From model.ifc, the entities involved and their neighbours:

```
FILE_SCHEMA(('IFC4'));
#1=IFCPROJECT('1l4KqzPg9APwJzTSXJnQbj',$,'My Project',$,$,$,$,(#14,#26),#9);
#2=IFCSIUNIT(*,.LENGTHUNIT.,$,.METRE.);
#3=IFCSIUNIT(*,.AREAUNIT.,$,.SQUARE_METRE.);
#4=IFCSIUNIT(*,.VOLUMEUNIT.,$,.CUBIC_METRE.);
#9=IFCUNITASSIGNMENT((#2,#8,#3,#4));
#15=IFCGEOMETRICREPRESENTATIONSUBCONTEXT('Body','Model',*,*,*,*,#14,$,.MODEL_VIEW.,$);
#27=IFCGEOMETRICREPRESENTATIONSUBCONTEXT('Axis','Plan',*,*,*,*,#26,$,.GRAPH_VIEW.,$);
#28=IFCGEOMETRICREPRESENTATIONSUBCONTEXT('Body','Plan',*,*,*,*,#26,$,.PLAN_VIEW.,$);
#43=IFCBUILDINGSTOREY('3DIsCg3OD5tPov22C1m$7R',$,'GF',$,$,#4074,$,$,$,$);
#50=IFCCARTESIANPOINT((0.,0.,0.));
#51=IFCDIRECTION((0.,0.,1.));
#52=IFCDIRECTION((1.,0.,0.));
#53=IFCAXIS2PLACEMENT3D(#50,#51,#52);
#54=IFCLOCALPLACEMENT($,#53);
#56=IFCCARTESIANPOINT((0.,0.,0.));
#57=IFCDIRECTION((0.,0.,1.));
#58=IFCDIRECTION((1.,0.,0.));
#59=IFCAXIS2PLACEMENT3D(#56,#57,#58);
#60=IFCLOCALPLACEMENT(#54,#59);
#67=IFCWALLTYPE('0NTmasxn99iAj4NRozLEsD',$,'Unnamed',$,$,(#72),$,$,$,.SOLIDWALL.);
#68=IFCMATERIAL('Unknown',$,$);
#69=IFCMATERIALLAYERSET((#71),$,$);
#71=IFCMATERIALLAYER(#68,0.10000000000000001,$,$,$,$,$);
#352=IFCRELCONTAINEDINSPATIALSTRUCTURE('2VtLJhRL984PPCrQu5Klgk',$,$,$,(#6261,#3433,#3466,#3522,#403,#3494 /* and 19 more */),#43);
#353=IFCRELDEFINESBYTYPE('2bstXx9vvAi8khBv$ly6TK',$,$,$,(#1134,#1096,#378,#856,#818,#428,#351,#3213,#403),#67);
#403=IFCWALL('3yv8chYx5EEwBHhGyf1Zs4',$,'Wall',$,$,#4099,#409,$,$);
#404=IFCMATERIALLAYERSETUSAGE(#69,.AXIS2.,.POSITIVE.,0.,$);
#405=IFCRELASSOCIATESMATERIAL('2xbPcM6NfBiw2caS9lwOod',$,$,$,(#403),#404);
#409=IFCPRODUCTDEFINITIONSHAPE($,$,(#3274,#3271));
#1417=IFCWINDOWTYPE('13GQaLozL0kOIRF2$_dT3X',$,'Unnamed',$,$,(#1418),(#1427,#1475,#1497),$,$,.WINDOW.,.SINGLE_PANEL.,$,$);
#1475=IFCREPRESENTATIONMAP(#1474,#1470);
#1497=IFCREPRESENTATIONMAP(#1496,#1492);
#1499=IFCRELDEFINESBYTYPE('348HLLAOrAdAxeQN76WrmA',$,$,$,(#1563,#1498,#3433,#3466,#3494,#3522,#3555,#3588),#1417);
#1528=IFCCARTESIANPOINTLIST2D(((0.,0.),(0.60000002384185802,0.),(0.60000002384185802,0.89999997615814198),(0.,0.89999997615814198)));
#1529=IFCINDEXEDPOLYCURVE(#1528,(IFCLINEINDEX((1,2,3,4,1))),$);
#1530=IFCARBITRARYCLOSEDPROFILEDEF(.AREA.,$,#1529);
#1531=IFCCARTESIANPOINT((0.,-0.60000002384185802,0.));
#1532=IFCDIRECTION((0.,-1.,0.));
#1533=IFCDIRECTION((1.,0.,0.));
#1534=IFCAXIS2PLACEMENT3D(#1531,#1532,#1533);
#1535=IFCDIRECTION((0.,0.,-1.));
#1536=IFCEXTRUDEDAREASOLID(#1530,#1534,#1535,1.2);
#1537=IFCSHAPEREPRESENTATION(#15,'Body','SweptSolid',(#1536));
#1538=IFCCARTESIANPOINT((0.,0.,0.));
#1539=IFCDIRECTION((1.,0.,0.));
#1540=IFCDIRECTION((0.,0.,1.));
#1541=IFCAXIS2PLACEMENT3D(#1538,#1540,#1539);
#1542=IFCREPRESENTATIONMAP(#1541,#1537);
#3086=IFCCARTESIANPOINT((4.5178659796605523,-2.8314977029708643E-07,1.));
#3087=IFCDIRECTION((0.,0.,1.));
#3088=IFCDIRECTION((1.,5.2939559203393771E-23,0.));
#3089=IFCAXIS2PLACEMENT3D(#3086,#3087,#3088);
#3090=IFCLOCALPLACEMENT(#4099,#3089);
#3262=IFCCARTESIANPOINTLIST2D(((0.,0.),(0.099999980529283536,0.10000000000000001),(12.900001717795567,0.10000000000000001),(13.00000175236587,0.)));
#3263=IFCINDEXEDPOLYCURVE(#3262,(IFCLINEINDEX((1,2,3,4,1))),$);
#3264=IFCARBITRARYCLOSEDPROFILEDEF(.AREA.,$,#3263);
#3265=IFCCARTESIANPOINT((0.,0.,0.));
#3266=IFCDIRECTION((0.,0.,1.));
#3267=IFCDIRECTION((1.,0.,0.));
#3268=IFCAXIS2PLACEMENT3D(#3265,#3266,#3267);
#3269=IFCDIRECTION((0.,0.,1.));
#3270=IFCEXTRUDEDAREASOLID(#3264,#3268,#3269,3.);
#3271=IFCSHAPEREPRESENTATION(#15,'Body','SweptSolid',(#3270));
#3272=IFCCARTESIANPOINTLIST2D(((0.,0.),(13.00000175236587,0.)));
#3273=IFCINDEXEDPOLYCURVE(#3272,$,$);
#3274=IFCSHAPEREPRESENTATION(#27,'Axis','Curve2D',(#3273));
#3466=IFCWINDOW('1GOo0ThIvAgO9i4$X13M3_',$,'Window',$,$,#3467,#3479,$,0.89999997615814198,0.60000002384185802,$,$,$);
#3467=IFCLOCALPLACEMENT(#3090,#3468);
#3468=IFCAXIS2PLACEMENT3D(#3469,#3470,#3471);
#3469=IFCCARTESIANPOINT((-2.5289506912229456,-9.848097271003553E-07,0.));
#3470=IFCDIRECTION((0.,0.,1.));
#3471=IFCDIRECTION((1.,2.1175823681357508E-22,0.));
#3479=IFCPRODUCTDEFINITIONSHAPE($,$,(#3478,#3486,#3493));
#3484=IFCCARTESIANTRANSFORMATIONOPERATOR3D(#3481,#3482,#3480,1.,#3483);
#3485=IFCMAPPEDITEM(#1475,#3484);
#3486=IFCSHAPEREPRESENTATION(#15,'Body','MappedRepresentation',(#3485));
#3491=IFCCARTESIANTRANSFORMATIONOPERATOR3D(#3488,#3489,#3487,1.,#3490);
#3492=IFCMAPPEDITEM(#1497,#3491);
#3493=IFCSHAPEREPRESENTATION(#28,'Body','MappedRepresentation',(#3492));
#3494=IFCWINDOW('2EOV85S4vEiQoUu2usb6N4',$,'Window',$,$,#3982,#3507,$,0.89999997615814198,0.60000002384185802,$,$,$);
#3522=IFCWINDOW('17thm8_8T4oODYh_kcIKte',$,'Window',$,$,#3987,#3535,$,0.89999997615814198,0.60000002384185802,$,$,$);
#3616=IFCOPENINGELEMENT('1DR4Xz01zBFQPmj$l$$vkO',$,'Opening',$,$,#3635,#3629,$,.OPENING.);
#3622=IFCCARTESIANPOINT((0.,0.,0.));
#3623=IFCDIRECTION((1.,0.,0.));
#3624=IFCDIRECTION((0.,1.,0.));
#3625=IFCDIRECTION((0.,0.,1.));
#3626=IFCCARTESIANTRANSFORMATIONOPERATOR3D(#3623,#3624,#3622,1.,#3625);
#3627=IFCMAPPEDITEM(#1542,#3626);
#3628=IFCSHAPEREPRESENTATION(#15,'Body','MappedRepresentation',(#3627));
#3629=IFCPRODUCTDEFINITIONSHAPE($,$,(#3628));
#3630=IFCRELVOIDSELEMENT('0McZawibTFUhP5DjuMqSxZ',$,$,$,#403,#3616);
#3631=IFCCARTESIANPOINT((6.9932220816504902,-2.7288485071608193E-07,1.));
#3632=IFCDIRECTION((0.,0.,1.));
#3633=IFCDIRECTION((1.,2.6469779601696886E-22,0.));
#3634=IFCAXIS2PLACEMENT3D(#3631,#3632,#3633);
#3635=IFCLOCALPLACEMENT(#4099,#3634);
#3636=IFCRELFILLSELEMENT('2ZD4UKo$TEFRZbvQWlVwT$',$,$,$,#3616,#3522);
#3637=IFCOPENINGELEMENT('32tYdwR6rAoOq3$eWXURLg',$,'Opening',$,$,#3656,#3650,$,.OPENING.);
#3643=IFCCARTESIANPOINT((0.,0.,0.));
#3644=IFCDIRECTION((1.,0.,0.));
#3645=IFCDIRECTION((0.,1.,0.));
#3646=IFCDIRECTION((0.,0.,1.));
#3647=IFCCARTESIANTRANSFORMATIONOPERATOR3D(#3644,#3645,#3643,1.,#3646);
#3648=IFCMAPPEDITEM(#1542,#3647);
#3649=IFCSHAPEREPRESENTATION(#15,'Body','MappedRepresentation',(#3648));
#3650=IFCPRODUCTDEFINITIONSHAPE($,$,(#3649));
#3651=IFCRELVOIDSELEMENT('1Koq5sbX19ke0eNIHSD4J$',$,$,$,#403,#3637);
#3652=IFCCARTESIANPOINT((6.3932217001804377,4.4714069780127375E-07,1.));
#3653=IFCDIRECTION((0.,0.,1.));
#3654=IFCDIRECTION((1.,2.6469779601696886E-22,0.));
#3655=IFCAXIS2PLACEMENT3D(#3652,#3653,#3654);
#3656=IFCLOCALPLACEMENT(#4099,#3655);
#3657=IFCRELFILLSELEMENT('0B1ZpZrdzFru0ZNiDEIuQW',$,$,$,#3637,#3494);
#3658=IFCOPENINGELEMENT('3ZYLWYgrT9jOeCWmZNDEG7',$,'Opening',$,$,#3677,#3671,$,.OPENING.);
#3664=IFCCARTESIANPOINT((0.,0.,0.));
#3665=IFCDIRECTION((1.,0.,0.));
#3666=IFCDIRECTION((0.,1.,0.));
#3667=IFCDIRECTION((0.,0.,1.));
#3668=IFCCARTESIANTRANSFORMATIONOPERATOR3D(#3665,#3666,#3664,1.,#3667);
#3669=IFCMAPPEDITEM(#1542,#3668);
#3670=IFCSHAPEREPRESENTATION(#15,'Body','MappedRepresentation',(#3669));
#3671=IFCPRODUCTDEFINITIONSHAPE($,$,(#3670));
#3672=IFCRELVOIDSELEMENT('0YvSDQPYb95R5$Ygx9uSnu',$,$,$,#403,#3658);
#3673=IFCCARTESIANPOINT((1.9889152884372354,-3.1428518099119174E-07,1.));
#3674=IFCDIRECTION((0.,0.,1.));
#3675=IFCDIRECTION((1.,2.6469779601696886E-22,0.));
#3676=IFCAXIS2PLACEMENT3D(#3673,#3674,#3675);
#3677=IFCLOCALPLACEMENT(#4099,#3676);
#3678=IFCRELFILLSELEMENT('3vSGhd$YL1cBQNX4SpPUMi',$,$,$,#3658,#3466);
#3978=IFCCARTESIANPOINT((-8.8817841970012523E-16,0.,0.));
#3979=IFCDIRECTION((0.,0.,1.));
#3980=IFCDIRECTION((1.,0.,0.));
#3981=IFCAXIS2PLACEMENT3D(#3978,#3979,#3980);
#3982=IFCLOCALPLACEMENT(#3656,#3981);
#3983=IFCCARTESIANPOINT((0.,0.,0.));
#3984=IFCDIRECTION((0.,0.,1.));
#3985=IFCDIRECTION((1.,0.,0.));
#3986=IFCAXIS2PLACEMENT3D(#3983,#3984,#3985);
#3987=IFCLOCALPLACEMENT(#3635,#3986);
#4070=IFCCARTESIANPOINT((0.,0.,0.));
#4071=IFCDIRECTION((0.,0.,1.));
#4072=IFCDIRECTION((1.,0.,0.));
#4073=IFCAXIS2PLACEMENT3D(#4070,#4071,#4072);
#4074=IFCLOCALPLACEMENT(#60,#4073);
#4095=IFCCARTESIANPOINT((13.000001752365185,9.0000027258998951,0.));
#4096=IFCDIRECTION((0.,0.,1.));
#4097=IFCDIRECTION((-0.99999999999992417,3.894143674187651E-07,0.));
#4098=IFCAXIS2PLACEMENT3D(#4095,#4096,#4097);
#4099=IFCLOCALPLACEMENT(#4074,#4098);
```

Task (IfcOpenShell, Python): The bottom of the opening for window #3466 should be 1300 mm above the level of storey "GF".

```python
import numpy as np
import ifcopenshell
import ifcopenshell.api.geometry
import ifcopenshell.geom
import ifcopenshell.util.element
import ifcopenshell.util.placement
import ifcopenshell.util.shape
import ifcopenshell.util.unit

model = ifcopenshell.open("model.ifc")
unit_scale = ifcopenshell.util.unit.calculate_unit_scale(model)

window = model.by_guid("1GOo0ThIvAgO9i4$X13M3_")
opening = window.FillsVoids[0].RelatingOpeningElement
storey = ifcopenshell.util.element.get_container(window, ifc_class="IfcBuildingStorey")
level = ifcopenshell.util.placement.get_local_placement(storey.ObjectPlacement)[2, 3]

# The opening's origin need not be at the sill, so measure its lowest point.
shape = ifcopenshell.geom.create_shape(ifcopenshell.geom.settings(), opening)
bottom = ifcopenshell.util.shape.get_shape_bottom_elevation(shape, shape.geometry) / unit_scale
dz = level + 1.3 - bottom

shift = np.array([0.0, 0.0, dz])
# The window is not placed relative to its opening, so move both.
for product in (opening, window):
    matrix = ifcopenshell.util.placement.get_local_placement(product.ObjectPlacement)
    matrix[:3, 3] += shift
    ifcopenshell.api.geometry.edit_object_placement(model, product=product, matrix=matrix, is_si=False)

print(f"moved by {dz * unit_scale:+.3f} m")

model.write("model_updated.ifc")
```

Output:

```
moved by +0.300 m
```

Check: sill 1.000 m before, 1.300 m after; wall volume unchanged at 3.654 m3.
